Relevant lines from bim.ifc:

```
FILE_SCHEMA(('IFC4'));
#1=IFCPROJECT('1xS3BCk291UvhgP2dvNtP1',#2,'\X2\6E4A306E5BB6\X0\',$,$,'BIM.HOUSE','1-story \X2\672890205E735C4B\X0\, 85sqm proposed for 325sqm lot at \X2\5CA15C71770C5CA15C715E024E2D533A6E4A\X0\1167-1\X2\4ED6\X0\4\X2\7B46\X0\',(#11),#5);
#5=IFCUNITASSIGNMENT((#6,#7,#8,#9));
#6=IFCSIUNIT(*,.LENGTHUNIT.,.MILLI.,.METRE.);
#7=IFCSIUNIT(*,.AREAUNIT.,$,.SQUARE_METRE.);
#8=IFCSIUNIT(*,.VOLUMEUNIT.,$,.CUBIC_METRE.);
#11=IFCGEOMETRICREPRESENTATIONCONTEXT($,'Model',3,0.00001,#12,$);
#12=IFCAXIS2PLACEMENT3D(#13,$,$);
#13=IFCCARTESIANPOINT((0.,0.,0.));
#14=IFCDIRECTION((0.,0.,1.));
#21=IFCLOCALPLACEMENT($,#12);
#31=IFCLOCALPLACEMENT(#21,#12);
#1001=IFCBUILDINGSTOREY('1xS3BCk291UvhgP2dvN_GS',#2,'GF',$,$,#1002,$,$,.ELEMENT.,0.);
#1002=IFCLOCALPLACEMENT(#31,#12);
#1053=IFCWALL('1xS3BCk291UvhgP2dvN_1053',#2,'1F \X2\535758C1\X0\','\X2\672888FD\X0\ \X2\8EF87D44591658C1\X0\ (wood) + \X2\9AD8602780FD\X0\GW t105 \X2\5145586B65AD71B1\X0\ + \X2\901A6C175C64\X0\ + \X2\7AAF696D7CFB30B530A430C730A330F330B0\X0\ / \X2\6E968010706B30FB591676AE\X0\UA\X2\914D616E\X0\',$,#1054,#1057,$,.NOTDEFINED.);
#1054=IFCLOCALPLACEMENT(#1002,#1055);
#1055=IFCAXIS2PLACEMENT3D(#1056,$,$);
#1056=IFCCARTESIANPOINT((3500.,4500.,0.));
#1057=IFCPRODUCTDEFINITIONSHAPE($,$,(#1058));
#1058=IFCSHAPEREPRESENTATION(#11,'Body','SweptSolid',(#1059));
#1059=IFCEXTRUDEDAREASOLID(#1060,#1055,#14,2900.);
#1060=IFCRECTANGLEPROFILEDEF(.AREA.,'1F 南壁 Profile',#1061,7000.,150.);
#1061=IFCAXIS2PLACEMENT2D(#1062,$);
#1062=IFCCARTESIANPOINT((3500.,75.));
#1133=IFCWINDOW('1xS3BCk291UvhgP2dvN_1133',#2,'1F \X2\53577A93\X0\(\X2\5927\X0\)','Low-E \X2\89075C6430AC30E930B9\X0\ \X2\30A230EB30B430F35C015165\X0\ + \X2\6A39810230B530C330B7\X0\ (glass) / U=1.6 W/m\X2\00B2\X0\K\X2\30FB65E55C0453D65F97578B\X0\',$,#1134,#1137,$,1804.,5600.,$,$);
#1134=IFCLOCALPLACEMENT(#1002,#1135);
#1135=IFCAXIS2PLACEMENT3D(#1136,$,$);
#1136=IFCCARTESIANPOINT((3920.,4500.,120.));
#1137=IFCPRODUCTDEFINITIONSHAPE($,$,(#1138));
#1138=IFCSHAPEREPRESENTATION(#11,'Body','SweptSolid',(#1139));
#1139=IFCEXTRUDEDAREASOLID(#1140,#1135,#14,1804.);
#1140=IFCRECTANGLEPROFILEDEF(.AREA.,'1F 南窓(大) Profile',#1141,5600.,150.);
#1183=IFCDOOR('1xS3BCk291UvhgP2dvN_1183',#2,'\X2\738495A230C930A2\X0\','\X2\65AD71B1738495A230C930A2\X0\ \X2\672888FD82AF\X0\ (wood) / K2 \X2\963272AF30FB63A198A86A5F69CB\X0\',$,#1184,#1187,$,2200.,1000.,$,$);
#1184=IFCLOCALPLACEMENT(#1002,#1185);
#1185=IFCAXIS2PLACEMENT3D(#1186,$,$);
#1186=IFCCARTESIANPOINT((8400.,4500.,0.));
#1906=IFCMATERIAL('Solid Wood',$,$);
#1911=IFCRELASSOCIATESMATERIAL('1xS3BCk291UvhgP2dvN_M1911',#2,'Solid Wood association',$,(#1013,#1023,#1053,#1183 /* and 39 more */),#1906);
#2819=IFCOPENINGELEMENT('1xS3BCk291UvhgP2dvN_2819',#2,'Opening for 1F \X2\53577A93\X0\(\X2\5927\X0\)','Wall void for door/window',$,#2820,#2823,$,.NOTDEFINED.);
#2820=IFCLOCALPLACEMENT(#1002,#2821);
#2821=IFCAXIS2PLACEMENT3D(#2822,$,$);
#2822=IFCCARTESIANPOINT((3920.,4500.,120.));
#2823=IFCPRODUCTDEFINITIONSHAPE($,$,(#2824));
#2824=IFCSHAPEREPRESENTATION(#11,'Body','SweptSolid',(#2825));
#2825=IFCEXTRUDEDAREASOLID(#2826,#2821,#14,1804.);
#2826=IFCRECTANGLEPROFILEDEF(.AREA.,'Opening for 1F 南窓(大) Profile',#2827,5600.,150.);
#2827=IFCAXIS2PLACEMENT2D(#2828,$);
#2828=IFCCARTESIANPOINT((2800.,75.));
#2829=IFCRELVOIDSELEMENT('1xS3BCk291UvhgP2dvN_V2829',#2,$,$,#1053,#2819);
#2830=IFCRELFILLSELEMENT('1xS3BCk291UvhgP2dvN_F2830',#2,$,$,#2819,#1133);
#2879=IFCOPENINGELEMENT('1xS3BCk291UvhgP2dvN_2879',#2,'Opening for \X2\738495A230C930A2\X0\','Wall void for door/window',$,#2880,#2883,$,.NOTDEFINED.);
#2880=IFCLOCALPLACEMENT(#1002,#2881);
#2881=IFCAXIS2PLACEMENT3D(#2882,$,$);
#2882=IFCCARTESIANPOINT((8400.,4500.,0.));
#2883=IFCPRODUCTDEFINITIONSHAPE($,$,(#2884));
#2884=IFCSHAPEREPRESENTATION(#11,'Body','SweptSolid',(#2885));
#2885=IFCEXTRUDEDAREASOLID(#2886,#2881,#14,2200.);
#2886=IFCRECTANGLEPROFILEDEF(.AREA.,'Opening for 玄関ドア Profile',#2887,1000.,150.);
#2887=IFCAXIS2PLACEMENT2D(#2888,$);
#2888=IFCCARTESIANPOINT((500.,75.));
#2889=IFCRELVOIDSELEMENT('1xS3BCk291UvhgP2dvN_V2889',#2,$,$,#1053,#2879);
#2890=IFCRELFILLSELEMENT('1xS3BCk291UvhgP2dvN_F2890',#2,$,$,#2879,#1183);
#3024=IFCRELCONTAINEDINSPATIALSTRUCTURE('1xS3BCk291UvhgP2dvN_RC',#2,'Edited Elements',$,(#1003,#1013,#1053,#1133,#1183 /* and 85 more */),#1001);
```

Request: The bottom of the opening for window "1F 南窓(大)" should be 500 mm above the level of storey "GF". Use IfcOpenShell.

```python
import numpy as np
import ifcopenshell
import ifcopenshell.api.geometry
import ifcopenshell.geom
import ifcopenshell.util.element
import ifcopenshell.util.placement
import ifcopenshell.util.shape
import ifcopenshell.util.unit

model = ifcopenshell.open("bim.ifc")
unit_scale = ifcopenshell.util.unit.calculate_unit_scale(model)

window = model.by_id(1133)
opening = window.FillsVoids[0].RelatingOpeningElement
storey = ifcopenshell.util.element.get_container(window, ifc_class="IfcBuildingStorey")
level = ifcopenshell.util.placement.get_local_placement(storey.ObjectPlacement)[2, 3]

# The opening's origin need not be at the sill, so measure its lowest point.
shape = ifcopenshell.geom.create_shape(ifcopenshell.geom.settings(), opening)
bottom = ifcopenshell.util.shape.get_shape_bottom_elevation(shape, shape.geometry) / unit_scale
dz = level + 0.5 / unit_scale - bottom

shift = np.array([0.0, 0.0, dz])
# The window is not placed relative to its opening, so move both.
for product in (opening, window):
    matrix = ifcopenshell.util.placement.get_local_placement(product.ObjectPlacement)
    matrix[:3, 3] += shift
    ifcopenshell.api.geometry.edit_object_placement(model, product=product, matrix=matrix, is_si=False)

print(f"moved by {dz * unit_scale:+.3f} m")

model.write("bim_v2.ifc")
```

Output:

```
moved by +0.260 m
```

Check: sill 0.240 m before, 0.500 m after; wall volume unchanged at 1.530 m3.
